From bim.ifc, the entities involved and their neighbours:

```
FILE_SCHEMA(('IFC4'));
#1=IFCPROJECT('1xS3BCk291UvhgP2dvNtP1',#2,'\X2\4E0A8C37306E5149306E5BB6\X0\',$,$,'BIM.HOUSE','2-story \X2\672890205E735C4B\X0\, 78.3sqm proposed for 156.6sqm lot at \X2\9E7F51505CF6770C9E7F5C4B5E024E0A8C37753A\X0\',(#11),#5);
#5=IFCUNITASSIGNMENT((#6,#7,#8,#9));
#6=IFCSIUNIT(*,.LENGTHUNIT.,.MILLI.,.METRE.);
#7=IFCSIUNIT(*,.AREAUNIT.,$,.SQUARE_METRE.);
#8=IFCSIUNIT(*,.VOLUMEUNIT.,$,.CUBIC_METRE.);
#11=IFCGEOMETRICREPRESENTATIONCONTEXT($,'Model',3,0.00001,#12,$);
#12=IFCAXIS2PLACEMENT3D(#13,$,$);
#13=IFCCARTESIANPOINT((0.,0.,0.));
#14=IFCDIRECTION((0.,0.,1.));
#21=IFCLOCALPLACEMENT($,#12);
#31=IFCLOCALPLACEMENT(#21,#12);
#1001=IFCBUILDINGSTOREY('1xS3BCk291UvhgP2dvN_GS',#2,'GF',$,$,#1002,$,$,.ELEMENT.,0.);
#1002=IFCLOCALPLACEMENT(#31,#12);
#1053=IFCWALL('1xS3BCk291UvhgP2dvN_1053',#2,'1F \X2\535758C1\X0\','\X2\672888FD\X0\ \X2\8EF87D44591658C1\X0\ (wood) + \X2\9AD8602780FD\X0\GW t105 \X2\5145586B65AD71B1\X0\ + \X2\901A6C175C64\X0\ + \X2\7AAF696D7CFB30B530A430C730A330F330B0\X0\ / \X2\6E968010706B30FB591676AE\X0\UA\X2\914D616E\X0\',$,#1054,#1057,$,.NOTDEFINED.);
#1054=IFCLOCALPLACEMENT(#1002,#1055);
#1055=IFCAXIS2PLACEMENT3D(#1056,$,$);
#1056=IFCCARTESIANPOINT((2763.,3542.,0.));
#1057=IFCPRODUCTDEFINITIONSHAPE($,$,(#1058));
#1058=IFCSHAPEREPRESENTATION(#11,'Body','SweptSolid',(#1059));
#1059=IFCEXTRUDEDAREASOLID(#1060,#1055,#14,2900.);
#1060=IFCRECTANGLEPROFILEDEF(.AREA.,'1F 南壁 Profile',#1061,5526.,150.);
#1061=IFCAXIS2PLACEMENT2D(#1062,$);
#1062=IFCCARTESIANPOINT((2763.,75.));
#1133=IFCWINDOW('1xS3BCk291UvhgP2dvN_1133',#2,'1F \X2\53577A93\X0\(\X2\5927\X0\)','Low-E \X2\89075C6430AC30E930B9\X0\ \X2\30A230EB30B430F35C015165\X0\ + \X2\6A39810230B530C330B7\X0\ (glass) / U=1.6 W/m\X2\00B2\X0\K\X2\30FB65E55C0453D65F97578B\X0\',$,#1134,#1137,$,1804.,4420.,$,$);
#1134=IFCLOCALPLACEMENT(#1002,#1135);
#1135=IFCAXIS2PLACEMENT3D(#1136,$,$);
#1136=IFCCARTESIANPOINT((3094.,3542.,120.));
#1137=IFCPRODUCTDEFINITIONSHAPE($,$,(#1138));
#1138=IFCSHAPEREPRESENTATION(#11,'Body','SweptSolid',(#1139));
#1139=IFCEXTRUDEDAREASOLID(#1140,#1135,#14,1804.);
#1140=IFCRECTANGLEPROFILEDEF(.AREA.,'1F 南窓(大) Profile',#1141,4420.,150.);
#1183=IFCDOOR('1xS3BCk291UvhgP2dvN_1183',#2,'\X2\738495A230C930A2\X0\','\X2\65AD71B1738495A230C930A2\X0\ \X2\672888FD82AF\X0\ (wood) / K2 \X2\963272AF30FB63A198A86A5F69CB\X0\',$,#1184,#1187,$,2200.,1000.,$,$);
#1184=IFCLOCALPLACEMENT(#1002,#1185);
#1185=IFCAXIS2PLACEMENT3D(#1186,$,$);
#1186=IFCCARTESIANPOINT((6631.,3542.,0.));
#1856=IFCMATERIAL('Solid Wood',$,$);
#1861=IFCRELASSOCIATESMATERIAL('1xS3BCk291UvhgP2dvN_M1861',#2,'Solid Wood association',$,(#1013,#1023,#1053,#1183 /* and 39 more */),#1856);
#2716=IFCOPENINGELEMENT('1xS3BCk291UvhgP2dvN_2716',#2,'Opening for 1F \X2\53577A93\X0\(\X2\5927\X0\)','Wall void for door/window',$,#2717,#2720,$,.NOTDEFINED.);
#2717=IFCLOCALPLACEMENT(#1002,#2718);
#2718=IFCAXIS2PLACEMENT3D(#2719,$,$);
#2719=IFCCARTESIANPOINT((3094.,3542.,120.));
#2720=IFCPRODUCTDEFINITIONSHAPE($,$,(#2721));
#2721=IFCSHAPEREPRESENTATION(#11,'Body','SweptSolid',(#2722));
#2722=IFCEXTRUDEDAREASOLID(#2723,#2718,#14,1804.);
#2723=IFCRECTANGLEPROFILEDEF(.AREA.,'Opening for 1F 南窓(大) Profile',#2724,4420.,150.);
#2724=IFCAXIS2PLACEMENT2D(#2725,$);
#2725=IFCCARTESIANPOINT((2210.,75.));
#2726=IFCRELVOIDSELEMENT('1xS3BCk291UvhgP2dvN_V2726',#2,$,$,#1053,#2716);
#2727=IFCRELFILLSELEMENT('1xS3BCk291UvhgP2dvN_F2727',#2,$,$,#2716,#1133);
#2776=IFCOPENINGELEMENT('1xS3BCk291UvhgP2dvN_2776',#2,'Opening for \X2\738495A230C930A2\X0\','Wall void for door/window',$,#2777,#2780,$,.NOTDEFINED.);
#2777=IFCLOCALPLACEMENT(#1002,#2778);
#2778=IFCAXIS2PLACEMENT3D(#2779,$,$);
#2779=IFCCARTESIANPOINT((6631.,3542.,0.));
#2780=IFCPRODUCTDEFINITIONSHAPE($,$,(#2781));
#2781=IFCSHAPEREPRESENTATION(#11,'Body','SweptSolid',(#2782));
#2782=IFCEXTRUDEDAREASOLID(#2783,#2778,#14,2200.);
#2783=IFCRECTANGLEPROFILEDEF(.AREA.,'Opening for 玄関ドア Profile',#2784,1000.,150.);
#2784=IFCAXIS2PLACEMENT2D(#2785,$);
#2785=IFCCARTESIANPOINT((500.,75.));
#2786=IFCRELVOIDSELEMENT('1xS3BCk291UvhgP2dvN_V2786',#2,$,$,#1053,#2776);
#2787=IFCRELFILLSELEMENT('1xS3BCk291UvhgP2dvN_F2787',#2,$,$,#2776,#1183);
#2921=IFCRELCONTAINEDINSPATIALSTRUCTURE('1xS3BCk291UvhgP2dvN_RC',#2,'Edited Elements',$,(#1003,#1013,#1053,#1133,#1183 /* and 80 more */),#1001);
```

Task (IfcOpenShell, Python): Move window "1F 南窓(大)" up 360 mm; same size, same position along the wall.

```python
import numpy as np
import ifcopenshell
import ifcopenshell.api.geometry
import ifcopenshell.util.placement
import ifcopenshell.util.unit

model = ifcopenshell.open("bim.ifc")
unit_scale = ifcopenshell.util.unit.calculate_unit_scale(model)

window = model.by_guid("1xS3BCk291UvhgP2dvN_1133")
opening = window.FillsVoids[0].RelatingOpeningElement
dz = 360.0

shift = np.array([0.0, 0.0, dz])
# The window is not placed relative to its opening, so move both.
for product in (opening, window):
    matrix = ifcopenshell.util.placement.get_local_placement(product.ObjectPlacement)
    matrix[:3, 3] += shift
    ifcopenshell.api.geometry.edit_object_placement(model, product=product, matrix=matrix, is_si=False)

print(f"moved by {dz * unit_scale:+.3f} m")

model.write("bim_updated.ifc")
```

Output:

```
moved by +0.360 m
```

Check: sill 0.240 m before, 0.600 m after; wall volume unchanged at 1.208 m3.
